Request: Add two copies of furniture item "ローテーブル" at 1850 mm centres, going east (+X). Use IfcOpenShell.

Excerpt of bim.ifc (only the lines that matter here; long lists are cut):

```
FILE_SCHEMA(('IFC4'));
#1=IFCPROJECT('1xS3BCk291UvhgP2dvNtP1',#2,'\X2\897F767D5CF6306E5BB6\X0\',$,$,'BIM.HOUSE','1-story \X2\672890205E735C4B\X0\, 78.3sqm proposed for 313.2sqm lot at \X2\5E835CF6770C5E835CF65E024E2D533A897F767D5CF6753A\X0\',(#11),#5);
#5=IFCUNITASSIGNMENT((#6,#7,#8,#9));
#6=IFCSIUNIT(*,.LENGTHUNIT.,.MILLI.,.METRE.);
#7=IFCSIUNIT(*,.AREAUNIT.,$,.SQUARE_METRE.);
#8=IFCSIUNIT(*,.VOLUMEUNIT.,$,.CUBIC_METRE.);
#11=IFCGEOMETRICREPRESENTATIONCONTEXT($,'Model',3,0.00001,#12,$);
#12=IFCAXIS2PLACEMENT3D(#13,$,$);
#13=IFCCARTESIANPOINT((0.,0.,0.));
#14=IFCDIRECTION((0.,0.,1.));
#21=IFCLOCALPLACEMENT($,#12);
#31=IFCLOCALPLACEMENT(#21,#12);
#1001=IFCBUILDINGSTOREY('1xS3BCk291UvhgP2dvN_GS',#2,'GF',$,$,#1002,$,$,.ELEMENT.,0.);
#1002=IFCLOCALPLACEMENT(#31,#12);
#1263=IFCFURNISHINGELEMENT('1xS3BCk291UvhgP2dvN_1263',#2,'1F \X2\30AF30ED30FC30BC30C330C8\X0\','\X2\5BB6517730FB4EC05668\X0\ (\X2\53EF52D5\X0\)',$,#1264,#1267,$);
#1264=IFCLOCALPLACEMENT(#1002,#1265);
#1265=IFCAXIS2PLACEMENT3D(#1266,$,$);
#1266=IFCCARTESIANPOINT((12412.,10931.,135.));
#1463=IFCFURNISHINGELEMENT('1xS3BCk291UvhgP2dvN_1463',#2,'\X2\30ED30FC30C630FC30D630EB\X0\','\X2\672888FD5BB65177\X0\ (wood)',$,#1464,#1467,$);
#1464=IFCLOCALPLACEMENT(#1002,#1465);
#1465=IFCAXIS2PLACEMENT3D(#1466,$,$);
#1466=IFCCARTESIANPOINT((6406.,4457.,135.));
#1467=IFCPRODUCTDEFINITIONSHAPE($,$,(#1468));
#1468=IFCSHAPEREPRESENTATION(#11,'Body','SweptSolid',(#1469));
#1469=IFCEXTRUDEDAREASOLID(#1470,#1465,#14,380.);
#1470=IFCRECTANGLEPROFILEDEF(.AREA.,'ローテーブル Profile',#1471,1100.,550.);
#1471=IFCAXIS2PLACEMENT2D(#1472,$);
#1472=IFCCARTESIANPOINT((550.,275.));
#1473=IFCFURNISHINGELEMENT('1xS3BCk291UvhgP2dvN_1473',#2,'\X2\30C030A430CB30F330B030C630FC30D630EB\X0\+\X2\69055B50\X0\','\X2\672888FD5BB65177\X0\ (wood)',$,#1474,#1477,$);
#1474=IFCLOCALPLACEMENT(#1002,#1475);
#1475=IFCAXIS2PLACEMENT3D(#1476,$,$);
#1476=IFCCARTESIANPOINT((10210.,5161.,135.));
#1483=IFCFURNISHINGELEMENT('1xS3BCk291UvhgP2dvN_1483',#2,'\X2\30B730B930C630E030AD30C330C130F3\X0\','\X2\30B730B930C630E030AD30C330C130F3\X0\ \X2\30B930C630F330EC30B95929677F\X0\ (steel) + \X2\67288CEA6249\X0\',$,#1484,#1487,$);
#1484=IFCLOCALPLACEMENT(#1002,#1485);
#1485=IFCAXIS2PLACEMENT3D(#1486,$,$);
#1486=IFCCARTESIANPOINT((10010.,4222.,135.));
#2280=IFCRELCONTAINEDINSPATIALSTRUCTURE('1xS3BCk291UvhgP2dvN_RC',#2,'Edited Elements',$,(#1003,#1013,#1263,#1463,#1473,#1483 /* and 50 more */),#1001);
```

```python
import numpy as np
import ifcopenshell
import ifcopenshell.api.geometry
import ifcopenshell.api.root
import ifcopenshell.util.element
import ifcopenshell.util.placement

model = ifcopenshell.open("bim.ifc")


def reuse_history(source, copy):
    """copy_class also copies each property set's owner history, people and application; keep the originals."""
    for rel in copy.IsDefinedBy:
        if rel.is_a("IfcRelDefinesByProperties") and (history := rel.RelatingPropertyDefinition.OwnerHistory):
            rel.RelatingPropertyDefinition.OwnerHistory = source.OwnerHistory
            ifcopenshell.util.element.remove_deep2(model, history)


source = model.by_id(1463)
base = ifcopenshell.util.placement.get_local_placement(source.ObjectPlacement)
step = np.array([1.0, 0.0, 0.0]) * 1850.0

for i in range(1, 3):
    copy = ifcopenshell.api.root.copy_class(model, product=source)
    copy.Representation = ifcopenshell.util.element.copy_deep(
        model, source.Representation, exclude=["IfcGeometricRepresentationContext", "IfcRepresentationMap"]
    )
    reuse_history(source, copy)
    matrix = base.copy()
    matrix[:3, 3] += i * step
    print("added at", matrix[:3, 3].round(3) + 0.0)
    ifcopenshell.api.geometry.edit_object_placement(model, product=copy, matrix=matrix, is_si=False)

model.write("bim_updated.ifc")
```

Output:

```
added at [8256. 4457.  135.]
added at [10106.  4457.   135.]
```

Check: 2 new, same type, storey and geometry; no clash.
